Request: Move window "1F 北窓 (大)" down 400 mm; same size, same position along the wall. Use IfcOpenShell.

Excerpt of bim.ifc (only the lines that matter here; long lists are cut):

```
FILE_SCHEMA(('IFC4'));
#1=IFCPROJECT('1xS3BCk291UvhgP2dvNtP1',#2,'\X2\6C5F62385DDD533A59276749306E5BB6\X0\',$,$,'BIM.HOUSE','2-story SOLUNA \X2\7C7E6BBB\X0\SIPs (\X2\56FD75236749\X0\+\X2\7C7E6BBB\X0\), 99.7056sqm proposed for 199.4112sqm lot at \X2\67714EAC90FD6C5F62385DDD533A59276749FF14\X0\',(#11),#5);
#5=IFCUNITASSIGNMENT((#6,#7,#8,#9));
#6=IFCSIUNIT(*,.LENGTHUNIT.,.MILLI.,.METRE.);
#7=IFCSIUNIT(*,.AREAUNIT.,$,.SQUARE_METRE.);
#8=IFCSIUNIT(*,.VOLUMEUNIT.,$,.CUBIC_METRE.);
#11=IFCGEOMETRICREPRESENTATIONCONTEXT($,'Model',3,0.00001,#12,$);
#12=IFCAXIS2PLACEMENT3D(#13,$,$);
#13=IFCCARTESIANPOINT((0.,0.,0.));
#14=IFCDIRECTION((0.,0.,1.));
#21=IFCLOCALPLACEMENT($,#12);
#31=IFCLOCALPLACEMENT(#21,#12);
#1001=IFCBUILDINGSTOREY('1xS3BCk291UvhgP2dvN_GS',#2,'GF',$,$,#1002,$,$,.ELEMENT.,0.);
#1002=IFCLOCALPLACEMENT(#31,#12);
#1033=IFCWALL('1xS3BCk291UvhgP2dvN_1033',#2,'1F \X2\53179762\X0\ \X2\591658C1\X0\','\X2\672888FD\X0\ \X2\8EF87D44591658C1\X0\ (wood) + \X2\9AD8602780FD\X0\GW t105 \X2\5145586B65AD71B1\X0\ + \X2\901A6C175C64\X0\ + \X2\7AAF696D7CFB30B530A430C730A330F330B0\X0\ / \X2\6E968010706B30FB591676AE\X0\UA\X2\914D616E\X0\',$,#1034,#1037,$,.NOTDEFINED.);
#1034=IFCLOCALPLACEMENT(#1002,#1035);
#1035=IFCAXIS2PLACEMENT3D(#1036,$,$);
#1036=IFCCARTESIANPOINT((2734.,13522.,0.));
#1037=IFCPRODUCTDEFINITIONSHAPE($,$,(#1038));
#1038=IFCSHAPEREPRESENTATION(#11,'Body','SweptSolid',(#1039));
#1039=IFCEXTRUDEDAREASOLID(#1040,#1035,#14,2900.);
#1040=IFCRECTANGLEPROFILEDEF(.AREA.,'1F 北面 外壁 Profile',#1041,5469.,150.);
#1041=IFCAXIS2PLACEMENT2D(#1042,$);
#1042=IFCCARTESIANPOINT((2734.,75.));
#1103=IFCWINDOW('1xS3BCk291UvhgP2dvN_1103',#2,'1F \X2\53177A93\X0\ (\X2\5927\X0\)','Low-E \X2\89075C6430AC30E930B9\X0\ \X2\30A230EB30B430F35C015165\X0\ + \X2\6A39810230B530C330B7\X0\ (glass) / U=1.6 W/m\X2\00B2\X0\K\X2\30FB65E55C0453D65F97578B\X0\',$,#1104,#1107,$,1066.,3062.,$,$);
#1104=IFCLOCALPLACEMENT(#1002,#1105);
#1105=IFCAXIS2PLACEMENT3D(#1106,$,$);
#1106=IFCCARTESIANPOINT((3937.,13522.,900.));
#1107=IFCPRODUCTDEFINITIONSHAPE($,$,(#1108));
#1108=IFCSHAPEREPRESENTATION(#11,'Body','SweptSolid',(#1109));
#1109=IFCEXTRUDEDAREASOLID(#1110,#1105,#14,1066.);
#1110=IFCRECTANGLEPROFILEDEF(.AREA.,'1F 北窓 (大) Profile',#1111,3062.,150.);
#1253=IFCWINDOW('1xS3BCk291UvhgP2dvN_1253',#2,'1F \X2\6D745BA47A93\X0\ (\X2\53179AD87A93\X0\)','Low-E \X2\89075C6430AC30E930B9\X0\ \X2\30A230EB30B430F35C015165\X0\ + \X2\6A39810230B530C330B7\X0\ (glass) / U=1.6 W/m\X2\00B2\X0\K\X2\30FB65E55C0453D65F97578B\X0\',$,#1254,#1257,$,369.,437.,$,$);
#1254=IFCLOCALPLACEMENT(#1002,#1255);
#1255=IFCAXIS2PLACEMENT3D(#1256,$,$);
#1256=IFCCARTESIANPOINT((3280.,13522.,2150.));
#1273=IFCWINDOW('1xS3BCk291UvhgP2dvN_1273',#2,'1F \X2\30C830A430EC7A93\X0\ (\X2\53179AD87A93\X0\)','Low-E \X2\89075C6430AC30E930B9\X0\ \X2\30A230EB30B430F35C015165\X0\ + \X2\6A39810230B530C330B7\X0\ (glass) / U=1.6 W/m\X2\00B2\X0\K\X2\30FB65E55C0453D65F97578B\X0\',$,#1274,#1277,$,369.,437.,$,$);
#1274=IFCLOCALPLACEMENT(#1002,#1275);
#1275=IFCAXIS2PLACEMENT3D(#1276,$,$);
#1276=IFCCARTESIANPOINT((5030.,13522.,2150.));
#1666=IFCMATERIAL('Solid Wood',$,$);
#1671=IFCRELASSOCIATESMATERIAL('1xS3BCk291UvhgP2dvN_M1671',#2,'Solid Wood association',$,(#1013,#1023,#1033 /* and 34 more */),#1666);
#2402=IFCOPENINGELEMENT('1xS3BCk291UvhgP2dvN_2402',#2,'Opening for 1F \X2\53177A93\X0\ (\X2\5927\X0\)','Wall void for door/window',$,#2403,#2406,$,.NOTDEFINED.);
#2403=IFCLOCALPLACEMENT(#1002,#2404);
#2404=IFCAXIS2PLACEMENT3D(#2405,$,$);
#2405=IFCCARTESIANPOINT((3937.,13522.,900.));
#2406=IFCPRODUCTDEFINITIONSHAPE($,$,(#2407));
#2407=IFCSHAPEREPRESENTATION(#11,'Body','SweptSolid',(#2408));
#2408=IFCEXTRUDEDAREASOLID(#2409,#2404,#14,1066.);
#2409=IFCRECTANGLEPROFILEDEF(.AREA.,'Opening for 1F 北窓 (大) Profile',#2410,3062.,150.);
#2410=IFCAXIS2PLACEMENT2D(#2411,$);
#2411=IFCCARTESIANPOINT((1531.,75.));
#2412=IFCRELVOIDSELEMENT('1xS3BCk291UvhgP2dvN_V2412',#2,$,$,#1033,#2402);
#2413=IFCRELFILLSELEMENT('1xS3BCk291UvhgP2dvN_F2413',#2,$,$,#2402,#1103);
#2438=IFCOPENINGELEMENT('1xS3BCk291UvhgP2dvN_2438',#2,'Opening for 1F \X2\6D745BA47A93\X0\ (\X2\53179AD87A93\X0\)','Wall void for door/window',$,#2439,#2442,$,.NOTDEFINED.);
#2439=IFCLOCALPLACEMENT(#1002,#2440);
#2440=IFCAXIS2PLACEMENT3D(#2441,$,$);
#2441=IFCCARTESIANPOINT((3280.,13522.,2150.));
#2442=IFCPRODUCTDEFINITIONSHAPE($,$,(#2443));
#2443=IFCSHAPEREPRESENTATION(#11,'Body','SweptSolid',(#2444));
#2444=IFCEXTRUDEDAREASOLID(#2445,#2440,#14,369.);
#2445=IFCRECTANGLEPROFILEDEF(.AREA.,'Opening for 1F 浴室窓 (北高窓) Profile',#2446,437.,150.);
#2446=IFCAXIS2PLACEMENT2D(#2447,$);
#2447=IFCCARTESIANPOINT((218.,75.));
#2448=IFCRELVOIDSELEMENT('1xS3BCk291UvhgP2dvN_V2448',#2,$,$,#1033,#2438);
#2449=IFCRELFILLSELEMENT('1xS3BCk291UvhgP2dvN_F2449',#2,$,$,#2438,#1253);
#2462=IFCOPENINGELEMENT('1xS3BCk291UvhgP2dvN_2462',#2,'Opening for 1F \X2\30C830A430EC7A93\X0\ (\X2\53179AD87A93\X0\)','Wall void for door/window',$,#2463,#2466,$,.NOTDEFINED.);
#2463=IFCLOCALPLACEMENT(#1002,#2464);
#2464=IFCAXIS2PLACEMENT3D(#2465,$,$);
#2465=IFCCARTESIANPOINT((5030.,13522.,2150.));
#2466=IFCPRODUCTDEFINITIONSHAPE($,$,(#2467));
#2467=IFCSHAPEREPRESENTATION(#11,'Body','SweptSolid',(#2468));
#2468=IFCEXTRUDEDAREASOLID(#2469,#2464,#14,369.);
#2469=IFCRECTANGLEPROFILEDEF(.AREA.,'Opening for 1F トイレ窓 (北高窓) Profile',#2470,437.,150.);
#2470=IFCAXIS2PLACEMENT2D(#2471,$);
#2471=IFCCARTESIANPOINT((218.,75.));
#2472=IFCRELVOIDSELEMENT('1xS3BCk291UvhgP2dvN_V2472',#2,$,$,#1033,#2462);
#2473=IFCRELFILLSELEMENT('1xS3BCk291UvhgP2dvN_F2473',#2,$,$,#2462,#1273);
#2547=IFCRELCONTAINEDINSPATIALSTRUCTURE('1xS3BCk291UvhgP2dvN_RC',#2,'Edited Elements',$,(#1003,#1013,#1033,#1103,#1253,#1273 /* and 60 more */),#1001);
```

```python
import numpy as np
import ifcopenshell
import ifcopenshell.api.geometry
import ifcopenshell.util.placement
import ifcopenshell.util.unit

model = ifcopenshell.open("bim.ifc")
unit_scale = ifcopenshell.util.unit.calculate_unit_scale(model)

window = model.by_guid("1xS3BCk291UvhgP2dvN_1103")
opening = window.FillsVoids[0].RelatingOpeningElement
dz = -400.0

shift = np.array([0.0, 0.0, dz])
# The window is not placed relative to its opening, so move both.
for product in (opening, window):
    matrix = ifcopenshell.util.placement.get_local_placement(product.ObjectPlacement)
    matrix[:3, 3] += shift
    ifcopenshell.api.geometry.edit_object_placement(model, product=product, matrix=matrix, is_si=False)

print(f"moved by {dz * unit_scale:+.3f} m")

model.write("bim_edited.ifc")
```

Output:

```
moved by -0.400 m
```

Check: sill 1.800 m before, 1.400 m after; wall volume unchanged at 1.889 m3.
